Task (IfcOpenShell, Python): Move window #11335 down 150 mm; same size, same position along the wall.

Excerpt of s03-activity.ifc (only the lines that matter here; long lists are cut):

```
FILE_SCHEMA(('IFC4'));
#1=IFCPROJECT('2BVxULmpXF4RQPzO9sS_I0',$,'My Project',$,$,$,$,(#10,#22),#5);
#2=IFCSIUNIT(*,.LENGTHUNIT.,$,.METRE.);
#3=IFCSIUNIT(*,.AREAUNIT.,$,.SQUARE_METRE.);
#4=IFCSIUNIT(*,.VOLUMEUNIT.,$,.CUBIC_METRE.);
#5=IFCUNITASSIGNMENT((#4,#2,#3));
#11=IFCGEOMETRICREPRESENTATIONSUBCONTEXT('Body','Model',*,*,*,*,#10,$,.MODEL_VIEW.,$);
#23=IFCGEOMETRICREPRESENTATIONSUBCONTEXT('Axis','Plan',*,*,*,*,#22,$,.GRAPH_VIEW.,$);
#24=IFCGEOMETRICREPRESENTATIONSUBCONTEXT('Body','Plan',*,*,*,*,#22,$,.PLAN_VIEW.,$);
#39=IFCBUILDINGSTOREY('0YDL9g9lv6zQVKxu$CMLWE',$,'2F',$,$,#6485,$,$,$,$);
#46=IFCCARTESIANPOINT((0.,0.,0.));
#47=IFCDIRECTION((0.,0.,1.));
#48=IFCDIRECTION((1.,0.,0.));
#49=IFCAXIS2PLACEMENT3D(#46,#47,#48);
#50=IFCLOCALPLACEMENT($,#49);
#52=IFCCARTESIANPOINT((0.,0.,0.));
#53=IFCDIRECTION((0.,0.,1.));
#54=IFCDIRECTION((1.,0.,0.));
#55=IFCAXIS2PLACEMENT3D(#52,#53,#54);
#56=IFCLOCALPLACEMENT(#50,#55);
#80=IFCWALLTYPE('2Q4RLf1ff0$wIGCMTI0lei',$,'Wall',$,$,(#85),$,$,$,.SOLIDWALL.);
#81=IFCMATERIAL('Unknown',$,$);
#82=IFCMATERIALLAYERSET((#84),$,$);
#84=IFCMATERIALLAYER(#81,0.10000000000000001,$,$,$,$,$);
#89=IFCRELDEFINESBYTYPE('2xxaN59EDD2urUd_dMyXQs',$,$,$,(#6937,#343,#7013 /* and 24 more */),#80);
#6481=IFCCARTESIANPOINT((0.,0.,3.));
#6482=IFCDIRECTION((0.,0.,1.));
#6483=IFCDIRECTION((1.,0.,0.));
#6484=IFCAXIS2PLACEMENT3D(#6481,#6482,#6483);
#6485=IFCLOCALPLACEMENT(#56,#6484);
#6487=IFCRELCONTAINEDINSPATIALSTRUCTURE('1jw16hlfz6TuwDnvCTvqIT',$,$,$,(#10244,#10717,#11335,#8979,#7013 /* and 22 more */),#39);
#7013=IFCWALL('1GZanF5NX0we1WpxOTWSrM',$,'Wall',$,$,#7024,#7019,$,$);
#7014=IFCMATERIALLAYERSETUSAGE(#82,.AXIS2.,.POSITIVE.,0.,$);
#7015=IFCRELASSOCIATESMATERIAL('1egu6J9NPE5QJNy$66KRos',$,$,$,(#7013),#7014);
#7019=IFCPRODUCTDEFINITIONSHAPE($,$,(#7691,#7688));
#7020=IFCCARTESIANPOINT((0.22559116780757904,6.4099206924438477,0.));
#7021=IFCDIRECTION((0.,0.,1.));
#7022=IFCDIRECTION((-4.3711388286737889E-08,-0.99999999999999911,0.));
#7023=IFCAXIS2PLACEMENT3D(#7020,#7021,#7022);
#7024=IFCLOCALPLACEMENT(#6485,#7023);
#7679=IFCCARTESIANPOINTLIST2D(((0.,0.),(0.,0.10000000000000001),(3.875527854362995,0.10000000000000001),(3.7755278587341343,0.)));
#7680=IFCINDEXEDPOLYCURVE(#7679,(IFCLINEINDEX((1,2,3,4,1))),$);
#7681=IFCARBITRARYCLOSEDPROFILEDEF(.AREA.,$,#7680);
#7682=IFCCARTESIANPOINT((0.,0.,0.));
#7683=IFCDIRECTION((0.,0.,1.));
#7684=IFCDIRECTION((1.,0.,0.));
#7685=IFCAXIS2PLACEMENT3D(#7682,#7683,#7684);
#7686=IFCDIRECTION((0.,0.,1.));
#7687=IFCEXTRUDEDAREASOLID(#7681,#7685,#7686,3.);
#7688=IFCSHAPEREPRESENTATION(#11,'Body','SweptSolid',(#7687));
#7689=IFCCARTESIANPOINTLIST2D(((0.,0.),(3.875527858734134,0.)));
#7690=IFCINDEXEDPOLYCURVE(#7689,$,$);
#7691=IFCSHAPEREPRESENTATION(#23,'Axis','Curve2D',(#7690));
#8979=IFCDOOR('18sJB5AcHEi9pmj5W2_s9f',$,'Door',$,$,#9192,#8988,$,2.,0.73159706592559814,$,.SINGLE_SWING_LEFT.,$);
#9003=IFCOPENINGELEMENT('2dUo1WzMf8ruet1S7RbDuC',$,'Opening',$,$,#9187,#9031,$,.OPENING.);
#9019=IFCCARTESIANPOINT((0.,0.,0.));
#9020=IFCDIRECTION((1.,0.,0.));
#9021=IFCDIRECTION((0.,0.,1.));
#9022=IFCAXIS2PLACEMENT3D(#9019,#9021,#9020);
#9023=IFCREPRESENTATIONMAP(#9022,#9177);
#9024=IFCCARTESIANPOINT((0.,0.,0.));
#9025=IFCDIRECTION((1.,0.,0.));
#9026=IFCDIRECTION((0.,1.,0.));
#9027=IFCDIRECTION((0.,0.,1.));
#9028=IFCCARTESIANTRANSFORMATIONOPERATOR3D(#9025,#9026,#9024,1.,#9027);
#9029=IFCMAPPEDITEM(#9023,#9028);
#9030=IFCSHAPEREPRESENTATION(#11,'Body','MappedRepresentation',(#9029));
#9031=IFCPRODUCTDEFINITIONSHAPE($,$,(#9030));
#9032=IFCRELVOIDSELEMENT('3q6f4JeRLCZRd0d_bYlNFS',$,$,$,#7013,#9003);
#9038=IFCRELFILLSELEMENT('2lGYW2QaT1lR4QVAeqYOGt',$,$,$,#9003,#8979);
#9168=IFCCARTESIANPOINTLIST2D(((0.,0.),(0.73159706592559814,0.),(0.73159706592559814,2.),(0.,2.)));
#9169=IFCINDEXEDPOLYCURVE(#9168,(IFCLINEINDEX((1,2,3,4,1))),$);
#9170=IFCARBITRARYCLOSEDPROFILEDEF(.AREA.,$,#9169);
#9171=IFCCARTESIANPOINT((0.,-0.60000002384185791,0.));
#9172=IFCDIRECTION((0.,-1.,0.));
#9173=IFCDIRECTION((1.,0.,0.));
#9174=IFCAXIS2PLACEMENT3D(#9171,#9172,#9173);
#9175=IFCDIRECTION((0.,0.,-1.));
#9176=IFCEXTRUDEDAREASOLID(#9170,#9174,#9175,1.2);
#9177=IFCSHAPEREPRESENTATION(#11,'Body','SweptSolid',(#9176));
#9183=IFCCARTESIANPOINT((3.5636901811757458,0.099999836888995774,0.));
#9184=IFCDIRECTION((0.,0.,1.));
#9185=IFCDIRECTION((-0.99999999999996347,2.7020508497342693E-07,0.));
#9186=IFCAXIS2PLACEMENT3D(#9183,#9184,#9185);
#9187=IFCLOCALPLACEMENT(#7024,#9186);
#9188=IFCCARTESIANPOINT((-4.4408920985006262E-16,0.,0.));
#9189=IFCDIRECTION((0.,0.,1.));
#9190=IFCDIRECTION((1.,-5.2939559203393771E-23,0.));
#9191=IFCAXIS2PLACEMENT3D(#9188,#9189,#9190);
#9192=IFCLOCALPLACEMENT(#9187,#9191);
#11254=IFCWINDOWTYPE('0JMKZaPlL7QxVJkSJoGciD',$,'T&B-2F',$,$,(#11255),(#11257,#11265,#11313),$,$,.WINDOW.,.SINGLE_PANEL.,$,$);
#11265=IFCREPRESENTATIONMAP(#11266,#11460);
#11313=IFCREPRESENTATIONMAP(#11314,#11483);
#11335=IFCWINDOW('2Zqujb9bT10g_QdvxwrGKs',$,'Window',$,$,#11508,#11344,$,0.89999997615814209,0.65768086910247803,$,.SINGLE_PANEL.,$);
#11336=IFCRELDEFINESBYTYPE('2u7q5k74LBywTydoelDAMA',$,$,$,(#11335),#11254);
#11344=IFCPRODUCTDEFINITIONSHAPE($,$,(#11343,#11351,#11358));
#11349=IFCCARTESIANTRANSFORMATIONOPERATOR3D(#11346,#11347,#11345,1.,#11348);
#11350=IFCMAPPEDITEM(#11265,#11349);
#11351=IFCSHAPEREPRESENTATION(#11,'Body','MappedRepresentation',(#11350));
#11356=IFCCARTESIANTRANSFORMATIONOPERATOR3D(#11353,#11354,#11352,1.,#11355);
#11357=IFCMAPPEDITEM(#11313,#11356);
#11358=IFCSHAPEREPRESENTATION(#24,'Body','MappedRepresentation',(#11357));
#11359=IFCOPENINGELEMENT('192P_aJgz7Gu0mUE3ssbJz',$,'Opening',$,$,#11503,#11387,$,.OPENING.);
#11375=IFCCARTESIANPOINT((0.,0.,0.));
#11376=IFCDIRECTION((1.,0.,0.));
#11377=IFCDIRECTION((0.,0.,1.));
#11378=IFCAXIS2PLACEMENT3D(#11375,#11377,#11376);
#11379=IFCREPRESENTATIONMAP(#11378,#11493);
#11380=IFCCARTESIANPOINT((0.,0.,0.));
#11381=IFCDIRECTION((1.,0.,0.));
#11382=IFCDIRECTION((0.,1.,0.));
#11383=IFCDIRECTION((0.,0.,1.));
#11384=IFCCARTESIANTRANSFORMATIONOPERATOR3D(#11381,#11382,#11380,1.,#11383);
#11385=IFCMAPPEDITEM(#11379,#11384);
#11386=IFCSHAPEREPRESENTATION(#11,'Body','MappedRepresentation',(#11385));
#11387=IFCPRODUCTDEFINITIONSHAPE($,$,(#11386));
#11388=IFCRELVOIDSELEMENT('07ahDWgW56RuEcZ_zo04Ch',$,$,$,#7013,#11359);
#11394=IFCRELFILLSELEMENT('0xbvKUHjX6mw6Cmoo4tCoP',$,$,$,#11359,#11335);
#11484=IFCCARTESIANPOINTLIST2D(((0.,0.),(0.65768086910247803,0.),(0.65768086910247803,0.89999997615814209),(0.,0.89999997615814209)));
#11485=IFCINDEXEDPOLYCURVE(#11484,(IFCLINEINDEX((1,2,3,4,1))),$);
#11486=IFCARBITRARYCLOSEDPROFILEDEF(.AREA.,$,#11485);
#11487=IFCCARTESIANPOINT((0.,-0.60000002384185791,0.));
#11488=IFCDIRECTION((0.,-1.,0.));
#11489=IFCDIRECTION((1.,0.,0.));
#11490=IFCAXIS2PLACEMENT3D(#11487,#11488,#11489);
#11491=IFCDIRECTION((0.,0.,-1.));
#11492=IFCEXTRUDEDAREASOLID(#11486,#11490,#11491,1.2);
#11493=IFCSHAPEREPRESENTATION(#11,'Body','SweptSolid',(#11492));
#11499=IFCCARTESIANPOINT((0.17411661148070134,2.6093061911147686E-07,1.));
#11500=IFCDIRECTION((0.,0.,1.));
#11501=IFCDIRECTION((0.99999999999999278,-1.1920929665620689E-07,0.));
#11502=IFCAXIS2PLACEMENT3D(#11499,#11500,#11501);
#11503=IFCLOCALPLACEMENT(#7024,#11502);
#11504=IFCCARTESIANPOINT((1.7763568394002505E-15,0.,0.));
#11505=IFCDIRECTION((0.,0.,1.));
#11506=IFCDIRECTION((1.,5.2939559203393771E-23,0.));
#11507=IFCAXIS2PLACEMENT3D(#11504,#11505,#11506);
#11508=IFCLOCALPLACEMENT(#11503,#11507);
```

```python
import numpy as np
import ifcopenshell
import ifcopenshell.api.geometry
import ifcopenshell.util.placement
import ifcopenshell.util.unit

model = ifcopenshell.open("s03-activity.ifc")
unit_scale = ifcopenshell.util.unit.calculate_unit_scale(model)

window = model.by_guid("2Zqujb9bT10g_QdvxwrGKs")
opening = window.FillsVoids[0].RelatingOpeningElement
dz = -0.15 / unit_scale

shift = np.array([0.0, 0.0, dz])
# The window is placed relative to its opening, so it follows when the opening moves.
matrix = ifcopenshell.util.placement.get_local_placement(opening.ObjectPlacement)
matrix[:3, 3] += shift
ifcopenshell.api.geometry.edit_object_placement(
    model, product=opening, matrix=matrix, is_si=False, should_transform_children=True
)

print(f"moved by {dz * unit_scale:+.3f} m")

model.write("s03-activity_v2.ifc")
```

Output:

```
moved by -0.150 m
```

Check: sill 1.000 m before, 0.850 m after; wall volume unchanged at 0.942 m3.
